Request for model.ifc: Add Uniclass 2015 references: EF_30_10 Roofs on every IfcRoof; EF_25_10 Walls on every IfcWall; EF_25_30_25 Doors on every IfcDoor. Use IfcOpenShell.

First a look at what the model holds.

```python
import ifcopenshell

model = ifcopenshell.open("model.ifc")
print(model.schema)
print("classifications:", [c.Name for c in model.by_type("IfcClassification")])
for ifc_class in ("IfcDoor", "IfcRoof", "IfcStair", "IfcWall", "IfcWindow"):
    print(ifc_class, len(model.by_type(ifc_class)))
```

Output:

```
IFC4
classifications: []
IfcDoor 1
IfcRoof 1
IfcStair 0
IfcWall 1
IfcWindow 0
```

```python
import ifcopenshell
import ifcopenshell.api.classification

model = ifcopenshell.open("model.ifc")

system = ifcopenshell.api.classification.add_classification(model, classification="Uniclass 2015")

codes = {
    "IfcRoof": ("EF_30_10", "Roofs"),
    "IfcWall": ("EF_25_10", "Walls"),
    "IfcDoor": ("EF_25_30_25", "Doors"),
}
for ifc_class, (code, name) in codes.items():
    products = model.by_type(ifc_class)
    ifcopenshell.api.classification.add_reference(
        model, products=products, classification=system, identification=code, name=name
    )
    print(code, len(products))

model.write("model_updated.ifc")
```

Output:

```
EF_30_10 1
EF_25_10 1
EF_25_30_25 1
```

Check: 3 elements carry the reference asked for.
